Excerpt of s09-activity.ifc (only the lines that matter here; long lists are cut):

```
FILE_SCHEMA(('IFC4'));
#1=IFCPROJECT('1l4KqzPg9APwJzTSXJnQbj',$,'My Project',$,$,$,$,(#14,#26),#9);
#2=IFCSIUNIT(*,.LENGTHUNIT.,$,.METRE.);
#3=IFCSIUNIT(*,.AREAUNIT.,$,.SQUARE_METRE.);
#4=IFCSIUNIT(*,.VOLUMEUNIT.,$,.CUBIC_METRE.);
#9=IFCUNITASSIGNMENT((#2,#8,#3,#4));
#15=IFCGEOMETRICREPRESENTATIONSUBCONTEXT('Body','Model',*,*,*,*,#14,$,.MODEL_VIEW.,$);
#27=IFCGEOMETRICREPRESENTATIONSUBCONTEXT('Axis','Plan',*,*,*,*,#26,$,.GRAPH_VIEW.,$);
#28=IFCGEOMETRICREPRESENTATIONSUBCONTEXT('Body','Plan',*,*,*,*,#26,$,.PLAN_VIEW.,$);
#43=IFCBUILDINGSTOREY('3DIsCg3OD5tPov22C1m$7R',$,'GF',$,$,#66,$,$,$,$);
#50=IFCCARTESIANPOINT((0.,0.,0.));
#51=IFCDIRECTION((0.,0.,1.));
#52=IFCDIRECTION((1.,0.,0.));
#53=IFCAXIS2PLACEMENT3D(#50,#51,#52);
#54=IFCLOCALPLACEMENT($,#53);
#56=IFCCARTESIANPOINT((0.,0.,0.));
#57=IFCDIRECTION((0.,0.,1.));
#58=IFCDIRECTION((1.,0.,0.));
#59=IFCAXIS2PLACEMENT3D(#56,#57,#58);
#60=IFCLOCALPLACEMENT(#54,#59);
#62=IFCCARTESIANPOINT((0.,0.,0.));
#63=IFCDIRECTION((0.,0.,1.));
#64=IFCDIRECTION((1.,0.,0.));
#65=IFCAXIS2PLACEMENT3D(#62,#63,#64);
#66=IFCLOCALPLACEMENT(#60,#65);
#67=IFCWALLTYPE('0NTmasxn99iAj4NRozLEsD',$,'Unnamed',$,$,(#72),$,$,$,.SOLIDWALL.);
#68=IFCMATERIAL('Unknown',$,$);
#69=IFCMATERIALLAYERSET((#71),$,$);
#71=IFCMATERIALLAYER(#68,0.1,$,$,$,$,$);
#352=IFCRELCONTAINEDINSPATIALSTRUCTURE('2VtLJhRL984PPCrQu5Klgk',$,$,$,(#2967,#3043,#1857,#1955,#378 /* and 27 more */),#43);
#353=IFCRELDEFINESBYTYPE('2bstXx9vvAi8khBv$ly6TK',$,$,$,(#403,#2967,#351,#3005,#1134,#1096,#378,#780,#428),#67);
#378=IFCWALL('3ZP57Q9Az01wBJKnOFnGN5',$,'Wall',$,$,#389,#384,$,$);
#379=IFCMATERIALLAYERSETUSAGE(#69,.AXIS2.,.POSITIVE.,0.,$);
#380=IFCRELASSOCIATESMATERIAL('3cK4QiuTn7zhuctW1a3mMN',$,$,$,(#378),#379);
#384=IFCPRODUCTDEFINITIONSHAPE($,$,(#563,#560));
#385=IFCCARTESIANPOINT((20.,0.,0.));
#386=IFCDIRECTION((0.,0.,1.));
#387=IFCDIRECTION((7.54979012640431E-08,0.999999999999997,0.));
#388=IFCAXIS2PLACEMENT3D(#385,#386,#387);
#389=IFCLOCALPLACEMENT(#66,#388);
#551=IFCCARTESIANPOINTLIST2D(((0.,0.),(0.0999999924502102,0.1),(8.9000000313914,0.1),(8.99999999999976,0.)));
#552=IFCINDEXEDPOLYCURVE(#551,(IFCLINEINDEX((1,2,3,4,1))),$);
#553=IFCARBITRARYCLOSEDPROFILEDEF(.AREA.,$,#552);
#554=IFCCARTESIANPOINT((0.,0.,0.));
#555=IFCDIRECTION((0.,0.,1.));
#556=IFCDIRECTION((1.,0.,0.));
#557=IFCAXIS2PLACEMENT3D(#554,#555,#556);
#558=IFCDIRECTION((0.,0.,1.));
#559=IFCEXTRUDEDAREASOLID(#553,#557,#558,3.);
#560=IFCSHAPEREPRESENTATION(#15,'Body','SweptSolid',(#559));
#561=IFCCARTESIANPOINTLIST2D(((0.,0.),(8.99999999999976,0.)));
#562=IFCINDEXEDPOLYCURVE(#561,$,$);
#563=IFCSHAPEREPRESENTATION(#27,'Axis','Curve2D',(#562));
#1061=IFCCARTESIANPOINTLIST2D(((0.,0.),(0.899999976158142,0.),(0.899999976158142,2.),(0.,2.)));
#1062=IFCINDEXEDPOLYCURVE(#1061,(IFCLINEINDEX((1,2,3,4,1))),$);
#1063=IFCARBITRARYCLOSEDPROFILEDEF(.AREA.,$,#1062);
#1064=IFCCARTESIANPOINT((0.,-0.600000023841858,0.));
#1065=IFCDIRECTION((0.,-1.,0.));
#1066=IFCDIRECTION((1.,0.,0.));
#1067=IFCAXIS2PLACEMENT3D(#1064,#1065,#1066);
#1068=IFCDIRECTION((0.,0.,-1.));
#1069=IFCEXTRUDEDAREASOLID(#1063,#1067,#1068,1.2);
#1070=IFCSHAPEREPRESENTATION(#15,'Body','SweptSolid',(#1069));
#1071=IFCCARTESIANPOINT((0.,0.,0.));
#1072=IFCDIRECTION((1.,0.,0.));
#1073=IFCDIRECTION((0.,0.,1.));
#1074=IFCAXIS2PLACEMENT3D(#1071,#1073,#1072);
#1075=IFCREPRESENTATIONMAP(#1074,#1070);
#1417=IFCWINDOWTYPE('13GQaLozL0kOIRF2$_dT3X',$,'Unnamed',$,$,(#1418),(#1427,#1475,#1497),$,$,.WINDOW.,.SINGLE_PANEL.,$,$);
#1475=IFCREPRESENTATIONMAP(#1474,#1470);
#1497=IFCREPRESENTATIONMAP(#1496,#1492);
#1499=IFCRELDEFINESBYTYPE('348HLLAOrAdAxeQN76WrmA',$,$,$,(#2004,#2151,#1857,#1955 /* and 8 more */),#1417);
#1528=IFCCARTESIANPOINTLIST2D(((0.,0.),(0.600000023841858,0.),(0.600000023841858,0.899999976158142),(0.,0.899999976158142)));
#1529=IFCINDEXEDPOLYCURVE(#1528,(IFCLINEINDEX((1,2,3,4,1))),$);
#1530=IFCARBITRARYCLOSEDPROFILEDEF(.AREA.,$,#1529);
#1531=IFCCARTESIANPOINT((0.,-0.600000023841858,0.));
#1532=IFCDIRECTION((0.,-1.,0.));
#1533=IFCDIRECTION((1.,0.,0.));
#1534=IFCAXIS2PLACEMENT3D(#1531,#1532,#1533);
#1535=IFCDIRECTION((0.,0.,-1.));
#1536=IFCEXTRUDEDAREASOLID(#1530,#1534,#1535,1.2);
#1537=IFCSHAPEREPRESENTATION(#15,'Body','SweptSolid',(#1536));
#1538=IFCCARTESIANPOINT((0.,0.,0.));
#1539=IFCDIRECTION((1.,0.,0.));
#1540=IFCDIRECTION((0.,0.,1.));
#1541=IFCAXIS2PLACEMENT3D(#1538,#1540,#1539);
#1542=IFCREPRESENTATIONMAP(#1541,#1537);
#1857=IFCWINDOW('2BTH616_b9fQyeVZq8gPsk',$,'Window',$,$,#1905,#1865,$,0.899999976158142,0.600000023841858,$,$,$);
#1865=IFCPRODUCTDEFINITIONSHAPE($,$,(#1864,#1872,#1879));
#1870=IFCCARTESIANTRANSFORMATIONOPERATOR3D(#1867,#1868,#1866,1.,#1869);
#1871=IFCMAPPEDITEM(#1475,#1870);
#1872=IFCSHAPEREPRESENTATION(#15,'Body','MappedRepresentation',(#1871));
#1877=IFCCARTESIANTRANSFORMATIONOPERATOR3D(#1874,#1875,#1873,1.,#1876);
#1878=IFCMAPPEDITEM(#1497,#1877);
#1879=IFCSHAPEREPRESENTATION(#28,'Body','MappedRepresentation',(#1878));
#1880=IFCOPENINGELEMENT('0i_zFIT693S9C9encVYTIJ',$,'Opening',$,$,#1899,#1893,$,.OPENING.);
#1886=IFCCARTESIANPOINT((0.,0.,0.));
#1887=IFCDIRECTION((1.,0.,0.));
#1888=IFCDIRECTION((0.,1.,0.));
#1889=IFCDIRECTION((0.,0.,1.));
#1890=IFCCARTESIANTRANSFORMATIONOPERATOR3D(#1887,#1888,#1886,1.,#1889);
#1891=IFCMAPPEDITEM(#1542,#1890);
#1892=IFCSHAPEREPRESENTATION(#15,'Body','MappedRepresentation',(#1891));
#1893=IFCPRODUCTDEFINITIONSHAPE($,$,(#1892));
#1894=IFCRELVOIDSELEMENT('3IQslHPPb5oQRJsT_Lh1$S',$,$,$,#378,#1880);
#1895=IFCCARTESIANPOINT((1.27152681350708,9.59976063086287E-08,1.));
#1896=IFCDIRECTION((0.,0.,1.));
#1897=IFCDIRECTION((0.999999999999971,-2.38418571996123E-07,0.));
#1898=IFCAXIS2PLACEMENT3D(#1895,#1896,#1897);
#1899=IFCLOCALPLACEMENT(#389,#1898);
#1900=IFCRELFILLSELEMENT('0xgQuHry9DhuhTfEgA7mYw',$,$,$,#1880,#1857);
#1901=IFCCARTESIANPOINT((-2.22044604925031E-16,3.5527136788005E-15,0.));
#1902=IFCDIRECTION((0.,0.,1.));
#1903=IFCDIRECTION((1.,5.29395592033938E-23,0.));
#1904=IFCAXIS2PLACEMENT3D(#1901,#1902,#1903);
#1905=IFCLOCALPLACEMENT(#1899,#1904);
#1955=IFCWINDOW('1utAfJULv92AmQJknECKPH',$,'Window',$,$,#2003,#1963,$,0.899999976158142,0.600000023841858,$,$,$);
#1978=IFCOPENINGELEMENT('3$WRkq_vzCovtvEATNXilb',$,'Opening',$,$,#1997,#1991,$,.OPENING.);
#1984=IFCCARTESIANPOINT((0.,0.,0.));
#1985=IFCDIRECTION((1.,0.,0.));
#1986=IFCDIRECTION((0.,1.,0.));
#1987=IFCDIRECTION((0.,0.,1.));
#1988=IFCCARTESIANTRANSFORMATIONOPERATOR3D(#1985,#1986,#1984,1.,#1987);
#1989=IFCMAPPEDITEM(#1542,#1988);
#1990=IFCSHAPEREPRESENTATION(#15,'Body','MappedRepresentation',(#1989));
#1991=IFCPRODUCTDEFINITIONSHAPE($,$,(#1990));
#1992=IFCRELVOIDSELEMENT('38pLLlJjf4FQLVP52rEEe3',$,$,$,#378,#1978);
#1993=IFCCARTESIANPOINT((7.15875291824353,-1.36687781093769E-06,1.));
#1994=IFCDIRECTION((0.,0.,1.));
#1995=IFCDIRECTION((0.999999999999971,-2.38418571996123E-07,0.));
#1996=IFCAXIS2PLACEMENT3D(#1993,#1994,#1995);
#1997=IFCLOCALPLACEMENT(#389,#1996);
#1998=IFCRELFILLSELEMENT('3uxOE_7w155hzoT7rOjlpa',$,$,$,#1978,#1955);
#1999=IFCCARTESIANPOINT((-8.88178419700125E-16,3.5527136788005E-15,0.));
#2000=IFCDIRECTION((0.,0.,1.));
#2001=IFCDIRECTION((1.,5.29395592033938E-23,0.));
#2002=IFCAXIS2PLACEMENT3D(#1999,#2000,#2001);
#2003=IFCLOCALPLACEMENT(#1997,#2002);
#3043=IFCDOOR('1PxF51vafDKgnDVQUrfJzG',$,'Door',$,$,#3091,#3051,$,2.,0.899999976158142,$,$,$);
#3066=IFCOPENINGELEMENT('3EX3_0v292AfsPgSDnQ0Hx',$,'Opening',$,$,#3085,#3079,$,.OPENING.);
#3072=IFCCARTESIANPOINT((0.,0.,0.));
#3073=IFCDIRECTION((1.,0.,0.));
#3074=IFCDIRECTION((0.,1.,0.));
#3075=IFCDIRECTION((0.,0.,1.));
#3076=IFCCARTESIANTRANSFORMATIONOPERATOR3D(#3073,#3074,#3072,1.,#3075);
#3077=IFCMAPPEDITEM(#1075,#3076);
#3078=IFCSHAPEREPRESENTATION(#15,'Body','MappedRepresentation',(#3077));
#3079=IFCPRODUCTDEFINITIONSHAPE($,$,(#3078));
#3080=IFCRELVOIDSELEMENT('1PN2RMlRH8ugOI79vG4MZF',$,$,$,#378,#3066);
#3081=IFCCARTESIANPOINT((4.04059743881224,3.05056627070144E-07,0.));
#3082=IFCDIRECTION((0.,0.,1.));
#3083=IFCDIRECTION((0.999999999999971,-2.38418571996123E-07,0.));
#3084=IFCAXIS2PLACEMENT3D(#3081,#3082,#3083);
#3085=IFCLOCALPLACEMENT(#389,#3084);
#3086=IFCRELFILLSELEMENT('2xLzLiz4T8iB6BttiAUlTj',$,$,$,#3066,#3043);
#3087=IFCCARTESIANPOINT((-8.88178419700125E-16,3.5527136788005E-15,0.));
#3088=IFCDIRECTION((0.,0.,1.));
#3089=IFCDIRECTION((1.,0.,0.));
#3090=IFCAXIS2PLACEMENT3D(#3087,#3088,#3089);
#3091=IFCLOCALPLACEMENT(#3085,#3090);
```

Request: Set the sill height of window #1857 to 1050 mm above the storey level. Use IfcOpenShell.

```python
import numpy as np
import ifcopenshell
import ifcopenshell.api.geometry
import ifcopenshell.geom
import ifcopenshell.util.element
import ifcopenshell.util.placement
import ifcopenshell.util.shape
import ifcopenshell.util.unit

model = ifcopenshell.open("s09-activity.ifc")
unit_scale = ifcopenshell.util.unit.calculate_unit_scale(model)

window = model.by_guid("2BTH616_b9fQyeVZq8gPsk")
opening = window.FillsVoids[0].RelatingOpeningElement
storey = ifcopenshell.util.element.get_container(window, ifc_class="IfcBuildingStorey")
level = ifcopenshell.util.placement.get_local_placement(storey.ObjectPlacement)[2, 3]

# The opening's origin need not be at the sill, so measure its lowest point.
shape = ifcopenshell.geom.create_shape(ifcopenshell.geom.settings(), opening)
bottom = ifcopenshell.util.shape.get_shape_bottom_elevation(shape, shape.geometry) / unit_scale
dz = level + 1.05 - bottom

shift = np.array([0.0, 0.0, dz])
# The window is placed relative to its opening, so it follows when the opening moves.
matrix = ifcopenshell.util.placement.get_local_placement(opening.ObjectPlacement)
matrix[:3, 3] += shift
ifcopenshell.api.geometry.edit_object_placement(
    model, product=opening, matrix=matrix, is_si=False, should_transform_children=True
)

print(f"moved by {dz * unit_scale:+.3f} m")

model.write("s09-activity_edited.ifc")
```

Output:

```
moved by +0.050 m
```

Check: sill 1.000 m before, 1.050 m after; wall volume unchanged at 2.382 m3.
